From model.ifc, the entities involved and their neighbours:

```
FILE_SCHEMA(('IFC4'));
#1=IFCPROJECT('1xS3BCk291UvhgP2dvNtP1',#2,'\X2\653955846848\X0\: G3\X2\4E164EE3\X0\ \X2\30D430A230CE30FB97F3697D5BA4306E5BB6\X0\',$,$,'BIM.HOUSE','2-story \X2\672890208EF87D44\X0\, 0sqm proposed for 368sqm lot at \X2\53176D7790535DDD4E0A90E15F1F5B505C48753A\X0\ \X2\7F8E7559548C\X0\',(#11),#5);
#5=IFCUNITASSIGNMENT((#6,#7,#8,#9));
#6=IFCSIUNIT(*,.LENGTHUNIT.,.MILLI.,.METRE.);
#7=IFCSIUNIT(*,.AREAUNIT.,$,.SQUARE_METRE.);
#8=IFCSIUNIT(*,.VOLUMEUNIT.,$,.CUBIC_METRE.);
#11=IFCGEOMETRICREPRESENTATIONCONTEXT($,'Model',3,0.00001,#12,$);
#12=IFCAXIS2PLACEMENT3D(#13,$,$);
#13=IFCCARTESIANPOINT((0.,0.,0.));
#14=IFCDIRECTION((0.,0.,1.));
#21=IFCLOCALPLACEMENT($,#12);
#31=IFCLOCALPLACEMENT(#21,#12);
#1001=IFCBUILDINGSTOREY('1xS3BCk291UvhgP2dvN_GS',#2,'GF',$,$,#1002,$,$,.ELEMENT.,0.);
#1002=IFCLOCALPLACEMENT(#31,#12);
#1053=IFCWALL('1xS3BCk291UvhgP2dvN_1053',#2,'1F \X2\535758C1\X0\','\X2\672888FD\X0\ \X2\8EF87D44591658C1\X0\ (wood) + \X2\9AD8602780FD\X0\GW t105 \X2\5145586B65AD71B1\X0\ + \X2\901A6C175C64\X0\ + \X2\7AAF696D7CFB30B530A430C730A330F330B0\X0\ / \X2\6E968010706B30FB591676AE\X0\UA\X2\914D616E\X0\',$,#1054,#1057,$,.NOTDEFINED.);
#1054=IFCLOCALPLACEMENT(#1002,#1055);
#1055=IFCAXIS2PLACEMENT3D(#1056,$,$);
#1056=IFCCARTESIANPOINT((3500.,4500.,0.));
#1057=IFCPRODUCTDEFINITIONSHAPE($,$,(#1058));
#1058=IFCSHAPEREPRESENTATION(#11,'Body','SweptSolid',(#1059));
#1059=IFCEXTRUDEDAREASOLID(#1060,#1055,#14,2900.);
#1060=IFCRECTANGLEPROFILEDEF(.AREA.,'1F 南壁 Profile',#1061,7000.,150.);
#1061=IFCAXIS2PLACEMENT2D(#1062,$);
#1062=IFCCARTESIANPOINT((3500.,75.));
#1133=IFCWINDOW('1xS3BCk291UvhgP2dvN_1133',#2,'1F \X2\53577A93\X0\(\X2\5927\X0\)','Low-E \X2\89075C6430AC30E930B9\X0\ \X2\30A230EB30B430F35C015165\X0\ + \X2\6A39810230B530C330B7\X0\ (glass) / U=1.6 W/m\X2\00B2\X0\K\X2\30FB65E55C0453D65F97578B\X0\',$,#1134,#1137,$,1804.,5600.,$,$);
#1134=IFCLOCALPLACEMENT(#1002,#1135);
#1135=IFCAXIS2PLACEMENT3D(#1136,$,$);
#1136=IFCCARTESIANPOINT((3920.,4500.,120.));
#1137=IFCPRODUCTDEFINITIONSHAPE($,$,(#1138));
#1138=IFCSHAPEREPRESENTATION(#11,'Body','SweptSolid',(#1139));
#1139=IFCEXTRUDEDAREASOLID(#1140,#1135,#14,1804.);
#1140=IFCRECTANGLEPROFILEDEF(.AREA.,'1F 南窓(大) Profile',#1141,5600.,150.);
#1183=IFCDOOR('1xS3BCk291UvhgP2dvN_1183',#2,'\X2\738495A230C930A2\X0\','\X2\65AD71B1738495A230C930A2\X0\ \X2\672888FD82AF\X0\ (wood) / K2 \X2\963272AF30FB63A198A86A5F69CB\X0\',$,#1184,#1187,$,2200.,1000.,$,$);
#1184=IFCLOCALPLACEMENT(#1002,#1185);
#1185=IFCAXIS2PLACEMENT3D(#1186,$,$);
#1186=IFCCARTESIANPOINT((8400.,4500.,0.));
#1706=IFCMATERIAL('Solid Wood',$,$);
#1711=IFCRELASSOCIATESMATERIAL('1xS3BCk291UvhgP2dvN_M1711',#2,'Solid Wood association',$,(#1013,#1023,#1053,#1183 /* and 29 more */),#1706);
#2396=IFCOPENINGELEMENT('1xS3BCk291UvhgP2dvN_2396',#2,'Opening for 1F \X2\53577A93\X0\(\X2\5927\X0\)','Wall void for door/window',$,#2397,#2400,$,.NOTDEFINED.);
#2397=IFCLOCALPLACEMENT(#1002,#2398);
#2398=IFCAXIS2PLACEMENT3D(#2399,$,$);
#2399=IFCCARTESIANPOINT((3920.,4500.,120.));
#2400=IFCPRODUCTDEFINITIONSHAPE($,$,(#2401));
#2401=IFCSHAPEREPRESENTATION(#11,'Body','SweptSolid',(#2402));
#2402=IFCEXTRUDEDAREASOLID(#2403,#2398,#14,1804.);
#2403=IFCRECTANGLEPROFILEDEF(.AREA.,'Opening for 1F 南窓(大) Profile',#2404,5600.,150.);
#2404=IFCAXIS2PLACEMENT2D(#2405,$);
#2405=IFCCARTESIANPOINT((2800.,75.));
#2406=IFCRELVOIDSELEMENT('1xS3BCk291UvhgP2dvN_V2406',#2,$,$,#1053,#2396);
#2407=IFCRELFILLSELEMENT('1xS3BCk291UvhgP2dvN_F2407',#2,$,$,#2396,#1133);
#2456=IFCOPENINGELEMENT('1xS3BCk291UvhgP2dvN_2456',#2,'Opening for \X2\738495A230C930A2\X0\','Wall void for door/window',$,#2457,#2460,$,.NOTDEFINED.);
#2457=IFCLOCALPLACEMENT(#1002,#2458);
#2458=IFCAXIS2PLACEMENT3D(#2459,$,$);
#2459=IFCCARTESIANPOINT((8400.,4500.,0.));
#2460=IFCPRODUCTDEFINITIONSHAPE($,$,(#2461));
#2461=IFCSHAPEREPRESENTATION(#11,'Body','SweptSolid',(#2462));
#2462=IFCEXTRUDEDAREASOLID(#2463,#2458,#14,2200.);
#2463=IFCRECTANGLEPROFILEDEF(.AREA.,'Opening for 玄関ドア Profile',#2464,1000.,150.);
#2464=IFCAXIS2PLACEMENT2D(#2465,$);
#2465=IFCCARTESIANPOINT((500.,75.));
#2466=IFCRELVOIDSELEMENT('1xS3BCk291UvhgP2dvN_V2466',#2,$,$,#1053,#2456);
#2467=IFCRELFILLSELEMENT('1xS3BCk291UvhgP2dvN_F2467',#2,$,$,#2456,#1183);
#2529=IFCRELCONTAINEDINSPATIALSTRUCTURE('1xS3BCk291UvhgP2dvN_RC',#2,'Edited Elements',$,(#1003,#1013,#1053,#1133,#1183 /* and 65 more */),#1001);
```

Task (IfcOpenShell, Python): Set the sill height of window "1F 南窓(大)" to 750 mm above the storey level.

```python
import numpy as np
import ifcopenshell
import ifcopenshell.api.geometry
import ifcopenshell.geom
import ifcopenshell.util.element
import ifcopenshell.util.placement
import ifcopenshell.util.shape
import ifcopenshell.util.unit

model = ifcopenshell.open("model.ifc")
unit_scale = ifcopenshell.util.unit.calculate_unit_scale(model)

window = model.by_id(1133)
opening = window.FillsVoids[0].RelatingOpeningElement
storey = ifcopenshell.util.element.get_container(window, ifc_class="IfcBuildingStorey")
level = ifcopenshell.util.placement.get_local_placement(storey.ObjectPlacement)[2, 3]

# The opening's origin need not be at the sill, so measure its lowest point.
shape = ifcopenshell.geom.create_shape(ifcopenshell.geom.settings(), opening)
bottom = ifcopenshell.util.shape.get_shape_bottom_elevation(shape, shape.geometry) / unit_scale
dz = level + 0.75 / unit_scale - bottom

shift = np.array([0.0, 0.0, dz])
# The window is not placed relative to its opening, so move both.
for product in (opening, window):
    matrix = ifcopenshell.util.placement.get_local_placement(product.ObjectPlacement)
    matrix[:3, 3] += shift
    ifcopenshell.api.geometry.edit_object_placement(model, product=product, matrix=matrix, is_si=False)

print(f"moved by {dz * unit_scale:+.3f} m")

model.write("model_v2.ifc")
```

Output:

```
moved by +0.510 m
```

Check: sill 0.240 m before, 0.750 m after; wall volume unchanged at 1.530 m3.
